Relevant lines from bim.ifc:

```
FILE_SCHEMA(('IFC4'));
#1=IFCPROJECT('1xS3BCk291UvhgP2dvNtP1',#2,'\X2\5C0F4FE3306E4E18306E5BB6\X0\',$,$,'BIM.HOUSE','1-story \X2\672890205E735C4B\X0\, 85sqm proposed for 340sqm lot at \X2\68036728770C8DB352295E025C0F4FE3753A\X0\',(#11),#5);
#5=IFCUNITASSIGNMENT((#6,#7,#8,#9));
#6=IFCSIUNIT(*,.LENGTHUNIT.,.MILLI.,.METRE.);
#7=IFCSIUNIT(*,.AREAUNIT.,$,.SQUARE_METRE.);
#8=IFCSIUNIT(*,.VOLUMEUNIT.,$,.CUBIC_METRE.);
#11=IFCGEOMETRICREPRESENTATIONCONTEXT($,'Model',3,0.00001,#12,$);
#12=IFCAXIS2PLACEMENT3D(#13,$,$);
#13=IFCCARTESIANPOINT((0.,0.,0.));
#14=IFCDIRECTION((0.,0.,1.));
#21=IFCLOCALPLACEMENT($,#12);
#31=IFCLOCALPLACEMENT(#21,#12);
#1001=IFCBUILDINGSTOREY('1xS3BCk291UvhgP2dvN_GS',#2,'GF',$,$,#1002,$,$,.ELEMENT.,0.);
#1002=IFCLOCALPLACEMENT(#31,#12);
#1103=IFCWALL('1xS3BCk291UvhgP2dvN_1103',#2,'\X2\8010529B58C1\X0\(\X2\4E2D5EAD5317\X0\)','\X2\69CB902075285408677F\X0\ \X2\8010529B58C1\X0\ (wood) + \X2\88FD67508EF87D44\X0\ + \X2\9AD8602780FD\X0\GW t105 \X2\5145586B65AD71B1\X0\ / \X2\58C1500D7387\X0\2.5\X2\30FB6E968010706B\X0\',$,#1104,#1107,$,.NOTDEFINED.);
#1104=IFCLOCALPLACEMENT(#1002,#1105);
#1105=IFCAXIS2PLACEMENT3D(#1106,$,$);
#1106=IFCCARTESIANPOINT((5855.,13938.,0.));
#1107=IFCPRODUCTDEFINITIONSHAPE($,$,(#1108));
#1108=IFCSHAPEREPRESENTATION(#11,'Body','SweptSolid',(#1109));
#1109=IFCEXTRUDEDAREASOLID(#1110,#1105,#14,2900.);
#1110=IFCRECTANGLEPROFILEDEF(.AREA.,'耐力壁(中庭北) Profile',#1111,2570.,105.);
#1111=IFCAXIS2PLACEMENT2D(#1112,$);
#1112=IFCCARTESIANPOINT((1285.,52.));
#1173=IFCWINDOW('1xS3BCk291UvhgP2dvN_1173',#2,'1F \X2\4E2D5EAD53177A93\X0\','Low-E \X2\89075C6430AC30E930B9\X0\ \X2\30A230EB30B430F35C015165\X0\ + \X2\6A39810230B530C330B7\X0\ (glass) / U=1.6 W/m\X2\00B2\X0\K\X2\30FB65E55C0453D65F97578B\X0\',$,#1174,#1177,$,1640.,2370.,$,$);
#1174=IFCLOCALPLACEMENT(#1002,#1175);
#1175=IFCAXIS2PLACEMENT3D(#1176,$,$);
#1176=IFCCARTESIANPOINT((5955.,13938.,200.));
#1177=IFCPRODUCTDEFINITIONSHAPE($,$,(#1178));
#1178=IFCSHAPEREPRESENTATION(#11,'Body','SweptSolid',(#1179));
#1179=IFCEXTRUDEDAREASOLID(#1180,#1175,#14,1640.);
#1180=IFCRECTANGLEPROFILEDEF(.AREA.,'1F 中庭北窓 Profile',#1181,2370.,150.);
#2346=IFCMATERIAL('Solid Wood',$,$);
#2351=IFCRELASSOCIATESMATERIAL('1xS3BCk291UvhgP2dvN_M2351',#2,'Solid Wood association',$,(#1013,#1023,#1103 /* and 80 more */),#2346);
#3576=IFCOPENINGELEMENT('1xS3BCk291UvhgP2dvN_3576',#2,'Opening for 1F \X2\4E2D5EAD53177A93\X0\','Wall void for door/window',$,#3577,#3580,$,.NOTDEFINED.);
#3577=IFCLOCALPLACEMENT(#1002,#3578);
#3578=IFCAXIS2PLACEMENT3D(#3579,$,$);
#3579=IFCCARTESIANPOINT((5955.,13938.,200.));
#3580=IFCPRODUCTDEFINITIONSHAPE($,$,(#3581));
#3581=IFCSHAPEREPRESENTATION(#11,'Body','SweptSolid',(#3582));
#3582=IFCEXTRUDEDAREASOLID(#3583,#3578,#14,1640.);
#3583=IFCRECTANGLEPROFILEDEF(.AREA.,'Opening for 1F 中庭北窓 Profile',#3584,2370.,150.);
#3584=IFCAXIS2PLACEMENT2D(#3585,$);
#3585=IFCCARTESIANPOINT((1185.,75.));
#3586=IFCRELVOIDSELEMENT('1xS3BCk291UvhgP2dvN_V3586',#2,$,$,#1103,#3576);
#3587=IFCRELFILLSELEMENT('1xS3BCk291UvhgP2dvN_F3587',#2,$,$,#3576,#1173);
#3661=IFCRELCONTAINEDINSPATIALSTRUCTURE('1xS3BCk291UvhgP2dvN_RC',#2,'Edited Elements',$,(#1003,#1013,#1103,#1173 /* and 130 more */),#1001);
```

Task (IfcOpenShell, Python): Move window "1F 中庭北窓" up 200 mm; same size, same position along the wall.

```python
import numpy as np
import ifcopenshell
import ifcopenshell.api.geometry
import ifcopenshell.util.placement
import ifcopenshell.util.unit

model = ifcopenshell.open("bim.ifc")
unit_scale = ifcopenshell.util.unit.calculate_unit_scale(model)

window = model.by_id(1173)
opening = window.FillsVoids[0].RelatingOpeningElement
dz = 0.2 / unit_scale

shift = np.array([0.0, 0.0, dz])
# The window is not placed relative to its opening, so move both.
for product in (opening, window):
    matrix = ifcopenshell.util.placement.get_local_placement(product.ObjectPlacement)
    matrix[:3, 3] += shift
    ifcopenshell.api.geometry.edit_object_placement(model, product=product, matrix=matrix, is_si=False)

print(f"moved by {dz * unit_scale:+.3f} m")

model.write("bim-out.ifc")
```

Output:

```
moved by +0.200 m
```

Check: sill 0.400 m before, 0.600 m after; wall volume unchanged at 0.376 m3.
